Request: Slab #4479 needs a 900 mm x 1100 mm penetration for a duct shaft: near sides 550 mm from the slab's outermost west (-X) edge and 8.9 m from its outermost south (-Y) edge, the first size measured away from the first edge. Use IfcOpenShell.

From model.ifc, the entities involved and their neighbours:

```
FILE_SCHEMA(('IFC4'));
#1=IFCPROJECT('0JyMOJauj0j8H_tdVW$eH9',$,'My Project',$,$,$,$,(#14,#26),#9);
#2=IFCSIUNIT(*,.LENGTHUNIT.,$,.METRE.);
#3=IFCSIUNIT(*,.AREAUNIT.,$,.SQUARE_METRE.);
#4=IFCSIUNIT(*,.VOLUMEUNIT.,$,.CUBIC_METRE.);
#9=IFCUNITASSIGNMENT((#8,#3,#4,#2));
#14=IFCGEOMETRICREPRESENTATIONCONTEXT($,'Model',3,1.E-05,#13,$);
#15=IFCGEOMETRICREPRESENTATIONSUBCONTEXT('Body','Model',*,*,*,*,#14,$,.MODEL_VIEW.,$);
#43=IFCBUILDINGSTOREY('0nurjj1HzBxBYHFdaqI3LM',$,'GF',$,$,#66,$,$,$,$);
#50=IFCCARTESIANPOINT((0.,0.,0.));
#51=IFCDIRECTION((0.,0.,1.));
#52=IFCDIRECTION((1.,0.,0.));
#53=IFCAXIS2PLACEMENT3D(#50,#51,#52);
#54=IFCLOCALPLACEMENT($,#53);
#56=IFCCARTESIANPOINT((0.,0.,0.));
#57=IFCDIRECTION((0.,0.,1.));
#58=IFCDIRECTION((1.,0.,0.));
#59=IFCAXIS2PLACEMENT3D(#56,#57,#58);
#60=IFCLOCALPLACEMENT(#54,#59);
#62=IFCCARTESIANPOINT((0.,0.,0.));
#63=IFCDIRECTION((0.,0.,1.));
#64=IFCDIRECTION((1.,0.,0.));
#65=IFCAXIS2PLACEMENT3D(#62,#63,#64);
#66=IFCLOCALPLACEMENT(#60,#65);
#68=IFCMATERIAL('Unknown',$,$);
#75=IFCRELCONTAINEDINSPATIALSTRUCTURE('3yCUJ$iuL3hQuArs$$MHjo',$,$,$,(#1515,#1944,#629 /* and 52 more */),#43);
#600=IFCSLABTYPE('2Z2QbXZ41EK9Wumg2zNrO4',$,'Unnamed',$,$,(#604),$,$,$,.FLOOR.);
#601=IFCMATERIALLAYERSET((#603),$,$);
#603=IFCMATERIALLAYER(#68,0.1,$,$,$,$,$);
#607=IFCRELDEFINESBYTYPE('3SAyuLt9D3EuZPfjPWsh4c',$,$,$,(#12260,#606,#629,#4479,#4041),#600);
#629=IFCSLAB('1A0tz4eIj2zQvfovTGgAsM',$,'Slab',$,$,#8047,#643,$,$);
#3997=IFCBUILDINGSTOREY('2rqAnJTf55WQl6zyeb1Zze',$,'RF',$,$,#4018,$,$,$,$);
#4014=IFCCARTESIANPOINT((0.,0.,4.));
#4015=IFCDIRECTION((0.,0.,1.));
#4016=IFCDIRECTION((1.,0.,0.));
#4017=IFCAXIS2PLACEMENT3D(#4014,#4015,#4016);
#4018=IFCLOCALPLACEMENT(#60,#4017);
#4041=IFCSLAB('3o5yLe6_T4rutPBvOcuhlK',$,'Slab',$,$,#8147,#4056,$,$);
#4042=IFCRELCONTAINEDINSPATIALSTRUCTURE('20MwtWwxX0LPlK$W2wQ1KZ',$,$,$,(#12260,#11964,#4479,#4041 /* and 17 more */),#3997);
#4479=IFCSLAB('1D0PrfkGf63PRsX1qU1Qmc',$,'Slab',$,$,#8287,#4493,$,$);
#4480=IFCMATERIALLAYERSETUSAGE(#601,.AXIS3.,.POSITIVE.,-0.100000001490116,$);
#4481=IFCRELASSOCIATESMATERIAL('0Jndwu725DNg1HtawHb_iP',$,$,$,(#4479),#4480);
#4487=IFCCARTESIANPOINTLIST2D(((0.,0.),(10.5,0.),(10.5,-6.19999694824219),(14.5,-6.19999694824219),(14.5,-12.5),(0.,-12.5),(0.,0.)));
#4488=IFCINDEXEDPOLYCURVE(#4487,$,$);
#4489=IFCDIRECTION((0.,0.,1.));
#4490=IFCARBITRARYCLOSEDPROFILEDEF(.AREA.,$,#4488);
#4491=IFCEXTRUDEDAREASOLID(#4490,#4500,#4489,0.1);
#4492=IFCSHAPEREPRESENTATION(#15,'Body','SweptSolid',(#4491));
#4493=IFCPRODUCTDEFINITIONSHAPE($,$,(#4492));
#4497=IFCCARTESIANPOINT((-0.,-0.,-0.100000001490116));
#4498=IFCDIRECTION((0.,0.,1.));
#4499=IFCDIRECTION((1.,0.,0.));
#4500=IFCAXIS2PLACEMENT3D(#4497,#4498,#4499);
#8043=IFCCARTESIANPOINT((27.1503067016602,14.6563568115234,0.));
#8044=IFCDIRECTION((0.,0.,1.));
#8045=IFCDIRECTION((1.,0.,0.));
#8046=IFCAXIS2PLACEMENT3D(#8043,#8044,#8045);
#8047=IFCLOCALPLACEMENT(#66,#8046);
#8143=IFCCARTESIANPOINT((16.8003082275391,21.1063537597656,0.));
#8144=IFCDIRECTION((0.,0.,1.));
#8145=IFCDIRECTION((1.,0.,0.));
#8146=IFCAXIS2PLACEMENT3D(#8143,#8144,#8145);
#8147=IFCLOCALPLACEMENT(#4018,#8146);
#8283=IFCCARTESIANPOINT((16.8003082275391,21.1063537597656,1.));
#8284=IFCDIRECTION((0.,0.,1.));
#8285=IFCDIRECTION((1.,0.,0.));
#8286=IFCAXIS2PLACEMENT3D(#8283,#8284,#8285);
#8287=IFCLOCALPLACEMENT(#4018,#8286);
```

```python
import numpy as np
import ifcopenshell
import ifcopenshell.api.feature
import ifcopenshell.api.geometry
import ifcopenshell.api.root
import ifcopenshell.geom
import ifcopenshell.util.placement
import ifcopenshell.util.representation
import ifcopenshell.util.shape
import ifcopenshell.util.unit

model = ifcopenshell.open("model.ifc")
unit_scale = ifcopenshell.util.unit.calculate_unit_scale(model)
settings = ifcopenshell.geom.settings()


def volume(element):
    """Net volume in cubic metres, openings subtracted."""
    shape = ifcopenshell.geom.create_shape(settings, element)
    return ifcopenshell.util.shape.get_volume(shape.geometry)


slab = model.by_id(4479)
before = volume(slab)

# Extent in the slab's own axes, in metres. The edges named are its -X and -Y sides.
slab_shape = ifcopenshell.geom.create_shape(settings, slab)
vertices = ifcopenshell.util.shape.get_vertices(slab_shape.geometry)
x_min, y_min, bottom = vertices.min(axis=0)
top = vertices[:, 2].max()

opening = ifcopenshell.api.root.create_entity(model, ifc_class="IfcOpeningElement", name="Duct shaft opening", predefined_type="OPENING")
context = ifcopenshell.util.representation.get_context(model, "Model", "Body", "MODEL_VIEW")
width, depth = 0.9, 1.1
outline = [(0.0, 0.0), (width, 0.0), (width, depth), (0.0, depth), (0.0, 0.0)]
# Overshoot both faces by 50 mm so the cut is clean.
shape = ifcopenshell.api.geometry.add_slab_representation(
    model, context=context, depth=top - bottom + 0.1, polyline=outline
)
ifcopenshell.api.geometry.assign_representation(model, product=opening, representation=shape)

matrix = ifcopenshell.util.placement.get_local_placement(slab.ObjectPlacement)
matrix[:, 3] = matrix @ np.append(np.array([x_min + 0.55, y_min + 8.9, bottom - 0.05]) / unit_scale, 1.0)
ifcopenshell.api.geometry.edit_object_placement(model, product=opening, matrix=matrix, is_si=False)
ifcopenshell.api.feature.add_feature(model, feature=opening, element=slab)

after = volume(slab)

print(f"slab volume {before:.3f} -> {after:.3f} m3")

model.write("model_v2.ifc")
```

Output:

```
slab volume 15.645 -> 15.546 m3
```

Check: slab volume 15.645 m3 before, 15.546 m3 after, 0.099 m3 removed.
